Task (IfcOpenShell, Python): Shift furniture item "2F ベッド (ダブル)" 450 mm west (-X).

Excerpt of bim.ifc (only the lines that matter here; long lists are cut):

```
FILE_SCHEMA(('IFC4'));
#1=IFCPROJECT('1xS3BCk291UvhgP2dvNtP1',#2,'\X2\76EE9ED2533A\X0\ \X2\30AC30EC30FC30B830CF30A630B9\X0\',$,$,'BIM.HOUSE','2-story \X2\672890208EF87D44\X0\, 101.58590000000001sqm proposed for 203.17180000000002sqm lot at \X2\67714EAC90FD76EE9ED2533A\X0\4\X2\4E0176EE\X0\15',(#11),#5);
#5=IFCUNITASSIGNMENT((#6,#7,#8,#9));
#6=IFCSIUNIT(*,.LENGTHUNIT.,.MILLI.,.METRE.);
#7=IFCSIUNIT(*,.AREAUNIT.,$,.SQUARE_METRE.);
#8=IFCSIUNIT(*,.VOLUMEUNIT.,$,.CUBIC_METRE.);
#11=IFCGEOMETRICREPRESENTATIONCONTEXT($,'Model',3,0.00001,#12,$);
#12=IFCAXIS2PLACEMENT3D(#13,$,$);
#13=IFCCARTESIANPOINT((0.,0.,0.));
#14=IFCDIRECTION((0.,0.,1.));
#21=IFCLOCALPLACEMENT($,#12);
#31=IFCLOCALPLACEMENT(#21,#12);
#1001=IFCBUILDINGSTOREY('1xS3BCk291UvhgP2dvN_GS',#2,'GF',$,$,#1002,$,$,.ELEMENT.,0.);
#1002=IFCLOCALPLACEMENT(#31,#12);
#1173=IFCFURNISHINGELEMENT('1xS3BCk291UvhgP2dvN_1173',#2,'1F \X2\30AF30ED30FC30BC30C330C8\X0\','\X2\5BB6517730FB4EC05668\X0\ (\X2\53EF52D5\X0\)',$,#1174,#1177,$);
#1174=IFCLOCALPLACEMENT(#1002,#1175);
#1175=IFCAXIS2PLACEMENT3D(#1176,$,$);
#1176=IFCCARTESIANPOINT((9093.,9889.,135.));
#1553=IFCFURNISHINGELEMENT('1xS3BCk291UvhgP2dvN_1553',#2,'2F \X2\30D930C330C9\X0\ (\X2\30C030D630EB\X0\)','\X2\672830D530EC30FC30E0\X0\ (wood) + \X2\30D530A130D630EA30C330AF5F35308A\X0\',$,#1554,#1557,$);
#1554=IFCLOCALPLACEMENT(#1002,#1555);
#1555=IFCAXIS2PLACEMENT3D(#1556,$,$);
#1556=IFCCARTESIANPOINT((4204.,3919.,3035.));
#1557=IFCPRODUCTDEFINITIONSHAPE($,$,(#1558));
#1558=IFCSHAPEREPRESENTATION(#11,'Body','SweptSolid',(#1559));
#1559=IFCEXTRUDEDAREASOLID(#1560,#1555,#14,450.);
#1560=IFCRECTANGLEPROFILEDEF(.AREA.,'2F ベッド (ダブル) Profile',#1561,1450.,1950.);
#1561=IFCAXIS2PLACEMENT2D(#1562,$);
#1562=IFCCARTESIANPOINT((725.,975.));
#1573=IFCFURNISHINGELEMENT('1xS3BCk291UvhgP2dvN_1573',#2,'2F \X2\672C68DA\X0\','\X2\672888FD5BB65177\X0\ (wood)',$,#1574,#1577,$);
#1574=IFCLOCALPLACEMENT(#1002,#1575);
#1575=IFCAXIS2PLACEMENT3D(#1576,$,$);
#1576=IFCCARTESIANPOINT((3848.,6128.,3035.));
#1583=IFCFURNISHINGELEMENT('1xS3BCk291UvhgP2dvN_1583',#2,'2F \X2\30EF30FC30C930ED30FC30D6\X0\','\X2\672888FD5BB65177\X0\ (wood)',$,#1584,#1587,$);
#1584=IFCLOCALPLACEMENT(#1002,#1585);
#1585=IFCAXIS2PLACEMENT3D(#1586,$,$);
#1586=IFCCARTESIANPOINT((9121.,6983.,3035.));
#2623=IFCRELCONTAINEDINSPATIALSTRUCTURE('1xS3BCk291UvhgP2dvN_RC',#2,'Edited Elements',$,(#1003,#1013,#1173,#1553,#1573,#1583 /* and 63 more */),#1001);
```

```python
import ifcopenshell
import ifcopenshell.api.geometry
import ifcopenshell.util.placement

model = ifcopenshell.open("bim.ifc")

item = model.by_id(1553)
matrix = ifcopenshell.util.placement.get_local_placement(item.ObjectPlacement)
matrix[0, 3] -= 450.0
ifcopenshell.api.geometry.edit_object_placement(model, product=item, matrix=matrix, is_si=False)

print(ifcopenshell.util.placement.get_local_placement(item.ObjectPlacement).round(3) + 0.0)

model.write("bim_v2.ifc")
```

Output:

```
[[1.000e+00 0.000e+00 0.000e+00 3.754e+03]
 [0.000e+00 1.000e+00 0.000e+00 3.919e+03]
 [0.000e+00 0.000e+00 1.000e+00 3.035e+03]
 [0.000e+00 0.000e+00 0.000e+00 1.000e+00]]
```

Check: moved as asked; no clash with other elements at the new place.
